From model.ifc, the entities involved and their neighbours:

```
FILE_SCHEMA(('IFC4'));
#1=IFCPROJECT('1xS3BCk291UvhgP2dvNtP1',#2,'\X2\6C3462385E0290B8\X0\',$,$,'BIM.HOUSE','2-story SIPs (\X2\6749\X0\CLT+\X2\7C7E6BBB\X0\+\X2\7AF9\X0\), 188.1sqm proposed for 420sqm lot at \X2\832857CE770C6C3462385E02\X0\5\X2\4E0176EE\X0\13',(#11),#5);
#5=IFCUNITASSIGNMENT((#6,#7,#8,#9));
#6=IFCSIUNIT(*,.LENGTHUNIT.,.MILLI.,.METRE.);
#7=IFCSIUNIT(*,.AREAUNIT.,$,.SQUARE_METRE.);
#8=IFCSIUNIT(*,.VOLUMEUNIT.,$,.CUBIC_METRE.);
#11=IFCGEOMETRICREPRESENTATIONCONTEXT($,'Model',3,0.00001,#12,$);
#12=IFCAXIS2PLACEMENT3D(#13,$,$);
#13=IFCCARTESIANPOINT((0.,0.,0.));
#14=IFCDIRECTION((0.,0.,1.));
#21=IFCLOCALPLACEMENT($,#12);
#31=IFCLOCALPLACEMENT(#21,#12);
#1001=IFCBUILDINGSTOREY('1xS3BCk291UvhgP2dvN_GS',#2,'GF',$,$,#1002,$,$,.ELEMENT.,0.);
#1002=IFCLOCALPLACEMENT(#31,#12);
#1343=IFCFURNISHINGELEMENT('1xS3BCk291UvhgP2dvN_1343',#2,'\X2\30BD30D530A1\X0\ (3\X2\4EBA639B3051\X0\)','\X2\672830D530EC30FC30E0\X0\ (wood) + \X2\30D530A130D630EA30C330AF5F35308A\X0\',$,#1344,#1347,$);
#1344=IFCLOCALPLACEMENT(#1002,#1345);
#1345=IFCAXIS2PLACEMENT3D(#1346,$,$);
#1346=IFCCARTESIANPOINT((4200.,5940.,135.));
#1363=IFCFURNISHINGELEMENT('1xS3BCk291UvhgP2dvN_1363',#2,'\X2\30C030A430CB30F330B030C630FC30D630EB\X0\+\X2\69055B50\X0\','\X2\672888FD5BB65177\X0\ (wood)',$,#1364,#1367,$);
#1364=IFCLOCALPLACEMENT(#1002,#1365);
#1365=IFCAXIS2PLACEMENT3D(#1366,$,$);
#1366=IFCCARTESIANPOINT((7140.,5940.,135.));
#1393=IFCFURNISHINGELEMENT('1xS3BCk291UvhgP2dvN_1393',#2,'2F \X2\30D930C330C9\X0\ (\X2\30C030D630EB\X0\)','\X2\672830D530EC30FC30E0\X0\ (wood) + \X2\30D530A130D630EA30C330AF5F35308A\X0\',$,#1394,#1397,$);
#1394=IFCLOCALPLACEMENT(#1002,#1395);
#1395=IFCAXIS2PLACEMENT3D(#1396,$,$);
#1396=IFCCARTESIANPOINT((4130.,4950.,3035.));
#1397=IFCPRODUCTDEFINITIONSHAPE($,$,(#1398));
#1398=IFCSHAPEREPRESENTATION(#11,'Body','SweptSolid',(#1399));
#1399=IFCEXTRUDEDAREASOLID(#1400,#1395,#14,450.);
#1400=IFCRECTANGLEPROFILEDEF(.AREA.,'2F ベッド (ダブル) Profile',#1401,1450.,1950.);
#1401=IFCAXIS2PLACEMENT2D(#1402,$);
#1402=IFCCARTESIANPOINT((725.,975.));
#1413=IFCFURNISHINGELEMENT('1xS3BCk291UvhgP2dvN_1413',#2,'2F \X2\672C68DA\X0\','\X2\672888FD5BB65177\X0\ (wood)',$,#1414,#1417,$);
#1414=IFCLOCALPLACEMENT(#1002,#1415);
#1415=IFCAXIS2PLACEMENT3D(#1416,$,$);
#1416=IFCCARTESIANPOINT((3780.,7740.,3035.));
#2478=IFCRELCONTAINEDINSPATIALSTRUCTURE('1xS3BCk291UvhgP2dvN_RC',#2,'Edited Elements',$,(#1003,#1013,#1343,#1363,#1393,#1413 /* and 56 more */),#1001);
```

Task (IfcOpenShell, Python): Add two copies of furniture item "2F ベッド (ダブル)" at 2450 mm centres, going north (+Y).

```python
import numpy as np
import ifcopenshell
import ifcopenshell.api.geometry
import ifcopenshell.api.root
import ifcopenshell.util.element
import ifcopenshell.util.placement
import ifcopenshell.util.unit

model = ifcopenshell.open("model.ifc")
unit_scale = ifcopenshell.util.unit.calculate_unit_scale(model)


def reuse_history(source, copy):
    """copy_class also copies each property set's owner history, people and application; keep the originals."""
    for rel in copy.IsDefinedBy:
        if rel.is_a("IfcRelDefinesByProperties") and (history := rel.RelatingPropertyDefinition.OwnerHistory):
            rel.RelatingPropertyDefinition.OwnerHistory = source.OwnerHistory
            ifcopenshell.util.element.remove_deep2(model, history)


source = model.by_guid("1xS3BCk291UvhgP2dvN_1393")
base = ifcopenshell.util.placement.get_local_placement(source.ObjectPlacement)
step = np.array([0.0, 1.0, 0.0]) * 2.45 / unit_scale

for i in range(1, 3):
    copy = ifcopenshell.api.root.copy_class(model, product=source)
    copy.Representation = ifcopenshell.util.element.copy_deep(
        model, source.Representation, exclude=["IfcGeometricRepresentationContext", "IfcRepresentationMap"]
    )
    reuse_history(source, copy)
    matrix = base.copy()
    matrix[:3, 3] += i * step
    print("added at", matrix[:3, 3].round(3) + 0.0)
    ifcopenshell.api.geometry.edit_object_placement(model, product=copy, matrix=matrix, is_si=False)

model.write("model_rev.ifc")
```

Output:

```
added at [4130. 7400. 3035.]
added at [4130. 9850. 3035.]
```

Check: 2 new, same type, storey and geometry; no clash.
